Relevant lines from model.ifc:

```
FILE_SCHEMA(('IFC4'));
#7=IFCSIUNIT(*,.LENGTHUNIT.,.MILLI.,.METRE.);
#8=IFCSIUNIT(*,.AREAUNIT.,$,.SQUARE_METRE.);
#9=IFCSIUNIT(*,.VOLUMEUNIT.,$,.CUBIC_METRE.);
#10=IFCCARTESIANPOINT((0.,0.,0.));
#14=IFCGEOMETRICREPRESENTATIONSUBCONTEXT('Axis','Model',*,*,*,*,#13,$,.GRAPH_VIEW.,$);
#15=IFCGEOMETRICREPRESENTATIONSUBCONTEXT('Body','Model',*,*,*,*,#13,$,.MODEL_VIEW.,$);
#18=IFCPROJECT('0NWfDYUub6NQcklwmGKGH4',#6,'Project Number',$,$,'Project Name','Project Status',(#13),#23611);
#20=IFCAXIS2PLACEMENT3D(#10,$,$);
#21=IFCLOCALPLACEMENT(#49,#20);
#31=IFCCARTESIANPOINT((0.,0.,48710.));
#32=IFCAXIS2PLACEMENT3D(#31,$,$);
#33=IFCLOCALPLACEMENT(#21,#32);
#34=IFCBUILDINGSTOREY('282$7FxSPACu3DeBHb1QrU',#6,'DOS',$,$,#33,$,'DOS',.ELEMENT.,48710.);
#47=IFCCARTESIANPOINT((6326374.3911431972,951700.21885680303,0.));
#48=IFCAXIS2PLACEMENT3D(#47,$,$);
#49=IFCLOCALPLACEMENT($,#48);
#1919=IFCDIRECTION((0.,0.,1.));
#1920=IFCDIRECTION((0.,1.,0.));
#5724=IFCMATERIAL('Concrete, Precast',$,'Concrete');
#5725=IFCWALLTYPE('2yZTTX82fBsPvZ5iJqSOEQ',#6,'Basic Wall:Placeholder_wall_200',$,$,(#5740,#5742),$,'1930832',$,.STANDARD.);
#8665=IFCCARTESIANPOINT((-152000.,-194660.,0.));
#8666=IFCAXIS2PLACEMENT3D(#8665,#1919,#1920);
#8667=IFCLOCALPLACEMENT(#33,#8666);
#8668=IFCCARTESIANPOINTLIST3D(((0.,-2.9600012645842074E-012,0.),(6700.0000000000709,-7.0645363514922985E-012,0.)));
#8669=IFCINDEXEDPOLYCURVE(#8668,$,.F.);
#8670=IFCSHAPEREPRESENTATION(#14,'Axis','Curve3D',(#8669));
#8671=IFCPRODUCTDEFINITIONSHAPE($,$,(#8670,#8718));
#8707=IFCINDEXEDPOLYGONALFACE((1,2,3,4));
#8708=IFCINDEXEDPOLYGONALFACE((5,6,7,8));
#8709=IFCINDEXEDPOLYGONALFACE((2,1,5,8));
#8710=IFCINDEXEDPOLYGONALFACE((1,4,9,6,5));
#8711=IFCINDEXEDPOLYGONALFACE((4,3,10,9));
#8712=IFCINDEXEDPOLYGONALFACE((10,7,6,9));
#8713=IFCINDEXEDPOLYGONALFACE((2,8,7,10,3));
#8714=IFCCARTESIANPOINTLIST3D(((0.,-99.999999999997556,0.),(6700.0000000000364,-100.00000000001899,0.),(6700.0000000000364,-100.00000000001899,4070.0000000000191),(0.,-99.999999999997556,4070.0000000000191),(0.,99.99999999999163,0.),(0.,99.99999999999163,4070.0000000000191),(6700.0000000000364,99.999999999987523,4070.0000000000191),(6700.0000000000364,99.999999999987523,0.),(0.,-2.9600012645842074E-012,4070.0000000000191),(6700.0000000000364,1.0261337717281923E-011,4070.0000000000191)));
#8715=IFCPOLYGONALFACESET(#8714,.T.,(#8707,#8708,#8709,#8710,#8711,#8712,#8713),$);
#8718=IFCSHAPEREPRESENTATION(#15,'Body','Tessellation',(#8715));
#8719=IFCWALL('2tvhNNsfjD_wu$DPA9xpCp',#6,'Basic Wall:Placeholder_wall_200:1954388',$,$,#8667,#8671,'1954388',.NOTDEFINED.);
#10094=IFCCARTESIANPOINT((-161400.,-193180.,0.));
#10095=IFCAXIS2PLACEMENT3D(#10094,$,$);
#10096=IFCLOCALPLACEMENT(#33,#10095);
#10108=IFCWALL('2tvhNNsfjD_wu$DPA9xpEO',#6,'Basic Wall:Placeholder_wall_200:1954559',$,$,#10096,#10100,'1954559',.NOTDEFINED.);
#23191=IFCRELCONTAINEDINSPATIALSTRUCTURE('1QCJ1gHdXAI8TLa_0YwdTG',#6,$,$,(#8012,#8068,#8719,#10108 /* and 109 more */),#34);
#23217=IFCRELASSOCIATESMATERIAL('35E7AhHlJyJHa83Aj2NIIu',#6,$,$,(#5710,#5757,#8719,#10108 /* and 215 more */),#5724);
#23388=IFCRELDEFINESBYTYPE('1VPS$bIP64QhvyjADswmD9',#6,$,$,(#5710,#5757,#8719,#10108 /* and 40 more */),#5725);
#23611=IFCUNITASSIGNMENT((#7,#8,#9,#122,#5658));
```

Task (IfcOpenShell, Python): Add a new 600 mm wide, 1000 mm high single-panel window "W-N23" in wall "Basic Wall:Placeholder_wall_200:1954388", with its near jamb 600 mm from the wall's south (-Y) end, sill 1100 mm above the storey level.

```python
import numpy as np
import ifcopenshell
import ifcopenshell.api.feature
import ifcopenshell.api.geometry
import ifcopenshell.api.root
import ifcopenshell.api.spatial
import ifcopenshell.geom
import ifcopenshell.util.element
import ifcopenshell.util.placement
import ifcopenshell.util.representation
import ifcopenshell.util.shape
import ifcopenshell.util.unit

model = ifcopenshell.open("model.ifc")
unit_scale = ifcopenshell.util.unit.calculate_unit_scale(model)
settings = ifcopenshell.geom.settings()


def volume(element):
    """Net volume in cubic metres, openings subtracted."""
    shape = ifcopenshell.geom.create_shape(settings, element)
    return ifcopenshell.util.shape.get_volume(shape.geometry)


wall = model.by_guid("2tvhNNsfjD_wu$DPA9xpCp")
storey = ifcopenshell.util.element.get_container(wall, ifc_class="IfcBuildingStorey")
context = ifcopenshell.util.representation.get_context(model, "Model", "Body", "MODEL_VIEW")
before = volume(wall)

width, height, from_end, sill = 0.6, 1, 0.6, 1.1  # metres

# The wall runs along its own X axis, and the end named is its -X end.
wall_shape = ifcopenshell.geom.create_shape(settings, wall)
x, y, z = ifcopenshell.util.shape.get_vertices(wall_shape.geometry).T
start = x.min() + from_end
face, thickness = float(y.min()), float(y.max() - y.min())
wall_matrix = ifcopenshell.util.placement.get_local_placement(wall.ObjectPlacement)
level = ifcopenshell.util.placement.get_local_placement(storey.ObjectPlacement)[2, 3]


def in_wall(x, y):
    """Placement at x, y metres in the wall's axes, at sill height."""
    matrix = wall_matrix.copy()
    matrix[:, 3] = wall_matrix @ np.array([x / unit_scale, y / unit_scale, 0.0, 1.0])
    matrix[2, 3] = level + sill / unit_scale
    return matrix


# Opening: a box that overshoots both wall faces by 50 mm.
opening = ifcopenshell.api.root.create_entity(model, ifc_class="IfcOpeningElement", predefined_type="OPENING")
box = ifcopenshell.api.geometry.add_wall_representation(
    model, context=context, length=width, height=height, thickness=thickness + 0.1
)
ifcopenshell.api.geometry.assign_representation(model, product=opening, representation=box)
ifcopenshell.api.geometry.edit_object_placement(model, product=opening, matrix=in_wall(start, face - 0.05), is_si=False)
ifcopenshell.api.feature.add_feature(model, feature=opening, element=wall)

window = ifcopenshell.api.root.create_entity(model, ifc_class="IfcWindow", name="W-N23", predefined_type="WINDOW")
window.OverallWidth, window.OverallHeight = width / unit_scale, height / unit_scale
window.PartitioningType = "SINGLE_PANEL"
body = ifcopenshell.api.geometry.add_window_representation(
    model,
    context=context,
    overall_width=window.OverallWidth,
    overall_height=window.OverallHeight,
    partition_type="SINGLE_PANEL",
)
ifcopenshell.api.geometry.assign_representation(model, product=window, representation=body)
ifcopenshell.api.spatial.assign_container(model, products=[window], relating_structure=storey)
ifcopenshell.api.feature.add_filling(model, opening=opening, element=window)

# Centre the window in the wall's thickness.
ifcopenshell.api.geometry.edit_object_placement(model, product=window, matrix=in_wall(start, face), is_si=False)
window_shape = ifcopenshell.geom.create_shape(settings, window)
depth = ifcopenshell.util.shape.get_vertices(window_shape.geometry)[:, 1]
offset = face + thickness / 2 - (depth.min() + depth.max()) / 2
ifcopenshell.api.geometry.edit_object_placement(model, product=window, matrix=in_wall(start, offset), is_si=False)

after = volume(wall)

print(f"wall volume {before:.3f} -> {after:.3f} m3")

model.write("model-out.ifc")
```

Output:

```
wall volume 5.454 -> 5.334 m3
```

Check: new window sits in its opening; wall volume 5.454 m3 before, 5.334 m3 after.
